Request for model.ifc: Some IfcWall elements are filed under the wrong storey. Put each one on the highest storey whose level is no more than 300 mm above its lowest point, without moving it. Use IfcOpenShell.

First a look at what the model holds.

```python
import ifcopenshell
import ifcopenshell.util.element
import ifcopenshell.util.placement

model = ifcopenshell.open("model.ifc")
print(model.schema)
for storey in model.by_type("IfcBuildingStorey"):
    level = ifcopenshell.util.placement.get_storey_elevation(storey)
    count = sum(e.is_a("IfcWall") for e in ifcopenshell.util.element.get_contained(storey))
    print(storey.id(), storey.Name, round(level, 3), count, sep=" | ")
```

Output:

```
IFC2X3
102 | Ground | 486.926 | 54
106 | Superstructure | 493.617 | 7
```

```python
import ifcopenshell
import ifcopenshell.api.spatial
import ifcopenshell.geom
import ifcopenshell.util.element
import ifcopenshell.util.placement
import ifcopenshell.util.shape
import ifcopenshell.util.unit

model = ifcopenshell.open("model.ifc")
unit_scale = ifcopenshell.util.unit.calculate_unit_scale(model)
settings = ifcopenshell.geom.settings()

levels = sorted(
    ((ifcopenshell.util.placement.get_storey_elevation(s) * unit_scale, s) for s in model.by_type("IfcBuildingStorey")),
    key=lambda pair: pair[0],
)

for e in model.by_type("IfcWall"):
    current = e.ContainedInStructure[0].RelatingStructure if e.ContainedInStructure else None
    if current is None or not current.is_a("IfcBuildingStorey"):
        continue
    shape = ifcopenshell.geom.create_shape(settings, e)
    bottom = ifcopenshell.util.shape.get_shape_bottom_elevation(shape, shape.geometry)
    below = [s for level, s in levels if level <= bottom + 0.3]
    storey = below[-1] if below else levels[0][1]
    if storey != current:
        # assign_container keeps the world position.
        ifcopenshell.api.spatial.assign_container(model, products=[e], relating_structure=storey)
        print(e.id(), current.Name, "->", storey.Name)

model.write("model_edited.ifc")
```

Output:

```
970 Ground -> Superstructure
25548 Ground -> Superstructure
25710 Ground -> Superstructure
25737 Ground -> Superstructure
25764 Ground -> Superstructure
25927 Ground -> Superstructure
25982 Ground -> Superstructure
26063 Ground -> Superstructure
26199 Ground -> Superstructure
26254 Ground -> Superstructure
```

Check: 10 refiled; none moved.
